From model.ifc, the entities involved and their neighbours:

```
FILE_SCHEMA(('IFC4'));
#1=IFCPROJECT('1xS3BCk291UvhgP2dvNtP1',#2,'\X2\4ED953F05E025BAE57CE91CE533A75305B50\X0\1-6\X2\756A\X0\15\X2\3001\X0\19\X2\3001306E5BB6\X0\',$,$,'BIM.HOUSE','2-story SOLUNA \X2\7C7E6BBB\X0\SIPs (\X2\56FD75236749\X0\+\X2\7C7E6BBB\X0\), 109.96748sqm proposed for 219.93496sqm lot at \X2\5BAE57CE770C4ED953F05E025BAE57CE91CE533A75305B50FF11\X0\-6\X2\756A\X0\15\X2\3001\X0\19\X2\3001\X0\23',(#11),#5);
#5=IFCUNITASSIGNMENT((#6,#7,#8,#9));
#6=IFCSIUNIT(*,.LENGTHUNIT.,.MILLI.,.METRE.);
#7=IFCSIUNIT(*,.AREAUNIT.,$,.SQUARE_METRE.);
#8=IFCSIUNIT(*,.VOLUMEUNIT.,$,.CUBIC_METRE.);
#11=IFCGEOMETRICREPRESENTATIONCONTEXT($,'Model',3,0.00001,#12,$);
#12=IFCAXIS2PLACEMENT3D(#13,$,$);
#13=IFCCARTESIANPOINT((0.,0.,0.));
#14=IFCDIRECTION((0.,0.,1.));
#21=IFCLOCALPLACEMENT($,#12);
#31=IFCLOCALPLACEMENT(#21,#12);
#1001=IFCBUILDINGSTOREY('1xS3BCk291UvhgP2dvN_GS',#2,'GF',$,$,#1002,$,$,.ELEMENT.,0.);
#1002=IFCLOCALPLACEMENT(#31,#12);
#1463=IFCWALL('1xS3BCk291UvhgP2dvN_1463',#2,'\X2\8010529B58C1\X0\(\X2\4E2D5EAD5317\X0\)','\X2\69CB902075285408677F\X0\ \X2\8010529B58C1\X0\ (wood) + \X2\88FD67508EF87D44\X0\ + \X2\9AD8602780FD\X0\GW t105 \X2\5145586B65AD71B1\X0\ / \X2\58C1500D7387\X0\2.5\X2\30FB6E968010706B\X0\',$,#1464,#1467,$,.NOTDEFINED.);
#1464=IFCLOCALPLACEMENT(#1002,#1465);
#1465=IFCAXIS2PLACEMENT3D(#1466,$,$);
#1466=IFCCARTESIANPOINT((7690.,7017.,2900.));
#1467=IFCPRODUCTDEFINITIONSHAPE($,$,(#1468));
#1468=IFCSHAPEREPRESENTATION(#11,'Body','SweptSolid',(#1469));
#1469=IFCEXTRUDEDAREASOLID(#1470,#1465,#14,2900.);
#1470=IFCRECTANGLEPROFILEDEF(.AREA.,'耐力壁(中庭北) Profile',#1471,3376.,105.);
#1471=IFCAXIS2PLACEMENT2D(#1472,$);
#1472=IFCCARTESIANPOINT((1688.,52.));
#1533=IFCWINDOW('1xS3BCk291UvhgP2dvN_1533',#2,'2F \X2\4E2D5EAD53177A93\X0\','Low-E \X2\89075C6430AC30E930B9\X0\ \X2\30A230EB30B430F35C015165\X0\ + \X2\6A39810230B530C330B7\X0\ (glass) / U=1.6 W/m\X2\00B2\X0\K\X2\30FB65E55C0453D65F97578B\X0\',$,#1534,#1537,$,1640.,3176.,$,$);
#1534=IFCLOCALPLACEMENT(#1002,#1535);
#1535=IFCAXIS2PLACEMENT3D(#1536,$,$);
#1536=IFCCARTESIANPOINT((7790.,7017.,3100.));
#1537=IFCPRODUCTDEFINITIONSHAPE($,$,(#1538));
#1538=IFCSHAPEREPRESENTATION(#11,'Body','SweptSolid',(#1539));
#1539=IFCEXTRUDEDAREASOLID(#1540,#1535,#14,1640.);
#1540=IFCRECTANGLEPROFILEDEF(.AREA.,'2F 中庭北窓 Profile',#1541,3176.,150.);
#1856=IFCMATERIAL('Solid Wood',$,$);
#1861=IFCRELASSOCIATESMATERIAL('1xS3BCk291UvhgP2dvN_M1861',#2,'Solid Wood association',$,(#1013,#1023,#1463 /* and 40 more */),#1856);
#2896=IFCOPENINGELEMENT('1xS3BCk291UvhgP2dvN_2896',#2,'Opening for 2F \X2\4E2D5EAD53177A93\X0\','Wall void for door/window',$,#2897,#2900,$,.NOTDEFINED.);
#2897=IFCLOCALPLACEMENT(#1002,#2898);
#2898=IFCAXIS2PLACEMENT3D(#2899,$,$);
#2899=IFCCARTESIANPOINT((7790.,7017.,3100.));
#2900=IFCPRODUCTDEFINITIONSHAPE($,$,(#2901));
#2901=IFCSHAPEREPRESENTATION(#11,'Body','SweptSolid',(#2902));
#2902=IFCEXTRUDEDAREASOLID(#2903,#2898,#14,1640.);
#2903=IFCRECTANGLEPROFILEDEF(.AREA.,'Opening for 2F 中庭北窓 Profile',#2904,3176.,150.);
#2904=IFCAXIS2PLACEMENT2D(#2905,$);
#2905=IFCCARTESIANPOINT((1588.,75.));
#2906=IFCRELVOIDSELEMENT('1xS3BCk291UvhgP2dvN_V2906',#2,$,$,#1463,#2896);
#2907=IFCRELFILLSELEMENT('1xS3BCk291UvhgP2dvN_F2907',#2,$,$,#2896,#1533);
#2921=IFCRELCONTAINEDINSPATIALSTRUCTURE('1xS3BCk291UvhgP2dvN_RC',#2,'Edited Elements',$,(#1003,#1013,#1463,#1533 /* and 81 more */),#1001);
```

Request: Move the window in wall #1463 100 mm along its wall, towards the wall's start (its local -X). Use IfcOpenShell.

```python
import ifcopenshell
import ifcopenshell.api.geometry
import ifcopenshell.util.placement
import ifcopenshell.util.unit

model = ifcopenshell.open("model.ifc")
unit_scale = ifcopenshell.util.unit.calculate_unit_scale(model)

window = model.by_guid("1xS3BCk291UvhgP2dvN_1533")
opening = window.FillsVoids[0].RelatingOpeningElement
wall = opening.VoidsElements[0].RelatingBuildingElement

wall_matrix = ifcopenshell.util.placement.get_local_placement(wall.ObjectPlacement)
shift = wall_matrix[:3, 0] * -0.1 / unit_scale
before = ifcopenshell.util.placement.get_local_placement(window.ObjectPlacement)[:3, 3].copy()

# The window is not placed relative to its opening, so move both.
for product in (opening, window):
    matrix = ifcopenshell.util.placement.get_local_placement(product.ObjectPlacement)
    matrix[:3, 3] += shift
    ifcopenshell.api.geometry.edit_object_placement(model, product=product, matrix=matrix, is_si=False)

after = ifcopenshell.util.placement.get_local_placement(window.ObjectPlacement)[:3, 3]
print("window moved by", (after - before).round(3) + 0.0)

model.write("model_updated.ifc")
```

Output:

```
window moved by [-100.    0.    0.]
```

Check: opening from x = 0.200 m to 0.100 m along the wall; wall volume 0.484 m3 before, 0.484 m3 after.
